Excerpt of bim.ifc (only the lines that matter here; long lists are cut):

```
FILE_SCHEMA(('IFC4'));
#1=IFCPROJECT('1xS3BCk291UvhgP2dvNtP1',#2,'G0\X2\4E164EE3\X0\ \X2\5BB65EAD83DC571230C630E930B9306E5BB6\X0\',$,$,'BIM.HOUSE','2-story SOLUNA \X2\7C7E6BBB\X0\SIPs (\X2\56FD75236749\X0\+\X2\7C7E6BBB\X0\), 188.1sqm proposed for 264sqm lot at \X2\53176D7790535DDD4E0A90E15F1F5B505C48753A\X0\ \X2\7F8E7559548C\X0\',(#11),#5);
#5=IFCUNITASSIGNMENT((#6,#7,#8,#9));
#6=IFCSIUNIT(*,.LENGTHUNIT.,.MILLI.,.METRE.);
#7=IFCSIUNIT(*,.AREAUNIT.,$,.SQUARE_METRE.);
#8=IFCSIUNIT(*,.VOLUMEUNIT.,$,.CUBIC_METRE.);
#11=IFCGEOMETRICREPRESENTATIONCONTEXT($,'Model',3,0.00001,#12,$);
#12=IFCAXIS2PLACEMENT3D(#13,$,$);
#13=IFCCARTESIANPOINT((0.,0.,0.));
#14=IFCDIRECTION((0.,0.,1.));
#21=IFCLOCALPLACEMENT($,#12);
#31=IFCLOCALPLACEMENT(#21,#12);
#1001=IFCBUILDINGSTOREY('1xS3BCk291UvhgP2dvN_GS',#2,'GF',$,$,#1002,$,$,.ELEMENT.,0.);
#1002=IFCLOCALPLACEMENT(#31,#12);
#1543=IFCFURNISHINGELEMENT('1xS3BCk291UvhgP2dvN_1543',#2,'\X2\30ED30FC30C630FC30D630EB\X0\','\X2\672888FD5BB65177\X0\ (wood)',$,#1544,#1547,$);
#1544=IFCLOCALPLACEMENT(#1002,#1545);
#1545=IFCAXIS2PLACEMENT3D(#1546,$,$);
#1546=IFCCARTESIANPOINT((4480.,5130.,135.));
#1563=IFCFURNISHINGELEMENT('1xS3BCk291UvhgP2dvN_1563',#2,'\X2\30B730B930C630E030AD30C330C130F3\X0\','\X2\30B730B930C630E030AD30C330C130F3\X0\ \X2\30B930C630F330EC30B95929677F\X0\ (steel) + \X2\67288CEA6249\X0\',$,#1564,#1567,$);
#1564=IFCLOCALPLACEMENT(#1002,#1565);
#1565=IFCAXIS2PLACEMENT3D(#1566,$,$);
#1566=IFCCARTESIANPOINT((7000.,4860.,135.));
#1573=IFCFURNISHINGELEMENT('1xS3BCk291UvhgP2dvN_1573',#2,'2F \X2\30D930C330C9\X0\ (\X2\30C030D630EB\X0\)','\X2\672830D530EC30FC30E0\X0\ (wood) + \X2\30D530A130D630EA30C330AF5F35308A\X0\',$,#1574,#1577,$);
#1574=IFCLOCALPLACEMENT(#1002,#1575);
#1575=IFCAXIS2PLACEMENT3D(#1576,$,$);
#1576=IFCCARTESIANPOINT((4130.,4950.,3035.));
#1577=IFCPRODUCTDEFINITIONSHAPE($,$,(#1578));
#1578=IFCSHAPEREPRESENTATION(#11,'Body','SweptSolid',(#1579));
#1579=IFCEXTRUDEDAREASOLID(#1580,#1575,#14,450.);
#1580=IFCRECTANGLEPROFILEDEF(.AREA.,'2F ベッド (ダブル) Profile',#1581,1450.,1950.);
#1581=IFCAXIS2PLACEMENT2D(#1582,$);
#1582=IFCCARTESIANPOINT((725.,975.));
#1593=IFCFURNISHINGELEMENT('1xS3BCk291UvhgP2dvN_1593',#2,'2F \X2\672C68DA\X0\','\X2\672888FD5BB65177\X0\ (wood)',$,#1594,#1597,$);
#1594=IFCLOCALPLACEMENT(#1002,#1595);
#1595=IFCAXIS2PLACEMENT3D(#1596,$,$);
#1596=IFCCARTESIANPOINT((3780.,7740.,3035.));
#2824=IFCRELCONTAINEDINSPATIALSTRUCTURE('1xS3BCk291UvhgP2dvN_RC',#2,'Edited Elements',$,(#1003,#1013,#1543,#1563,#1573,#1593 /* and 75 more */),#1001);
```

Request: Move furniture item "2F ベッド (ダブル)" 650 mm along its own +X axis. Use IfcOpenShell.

```python
import ifcopenshell
import ifcopenshell.api.geometry
import ifcopenshell.util.placement

model = ifcopenshell.open("bim.ifc")

item = model.by_id(1573)
matrix = ifcopenshell.util.placement.get_local_placement(item.ObjectPlacement)
matrix[:3, 3] += matrix[:3, 0] * 650.0
ifcopenshell.api.geometry.edit_object_placement(model, product=item, matrix=matrix, is_si=False)

print(ifcopenshell.util.placement.get_local_placement(item.ObjectPlacement).round(3) + 0.0)

model.write("bim_updated.ifc")
```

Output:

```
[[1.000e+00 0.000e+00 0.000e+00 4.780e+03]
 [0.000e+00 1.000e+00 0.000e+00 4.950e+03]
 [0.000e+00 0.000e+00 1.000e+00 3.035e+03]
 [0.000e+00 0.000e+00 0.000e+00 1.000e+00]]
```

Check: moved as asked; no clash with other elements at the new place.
